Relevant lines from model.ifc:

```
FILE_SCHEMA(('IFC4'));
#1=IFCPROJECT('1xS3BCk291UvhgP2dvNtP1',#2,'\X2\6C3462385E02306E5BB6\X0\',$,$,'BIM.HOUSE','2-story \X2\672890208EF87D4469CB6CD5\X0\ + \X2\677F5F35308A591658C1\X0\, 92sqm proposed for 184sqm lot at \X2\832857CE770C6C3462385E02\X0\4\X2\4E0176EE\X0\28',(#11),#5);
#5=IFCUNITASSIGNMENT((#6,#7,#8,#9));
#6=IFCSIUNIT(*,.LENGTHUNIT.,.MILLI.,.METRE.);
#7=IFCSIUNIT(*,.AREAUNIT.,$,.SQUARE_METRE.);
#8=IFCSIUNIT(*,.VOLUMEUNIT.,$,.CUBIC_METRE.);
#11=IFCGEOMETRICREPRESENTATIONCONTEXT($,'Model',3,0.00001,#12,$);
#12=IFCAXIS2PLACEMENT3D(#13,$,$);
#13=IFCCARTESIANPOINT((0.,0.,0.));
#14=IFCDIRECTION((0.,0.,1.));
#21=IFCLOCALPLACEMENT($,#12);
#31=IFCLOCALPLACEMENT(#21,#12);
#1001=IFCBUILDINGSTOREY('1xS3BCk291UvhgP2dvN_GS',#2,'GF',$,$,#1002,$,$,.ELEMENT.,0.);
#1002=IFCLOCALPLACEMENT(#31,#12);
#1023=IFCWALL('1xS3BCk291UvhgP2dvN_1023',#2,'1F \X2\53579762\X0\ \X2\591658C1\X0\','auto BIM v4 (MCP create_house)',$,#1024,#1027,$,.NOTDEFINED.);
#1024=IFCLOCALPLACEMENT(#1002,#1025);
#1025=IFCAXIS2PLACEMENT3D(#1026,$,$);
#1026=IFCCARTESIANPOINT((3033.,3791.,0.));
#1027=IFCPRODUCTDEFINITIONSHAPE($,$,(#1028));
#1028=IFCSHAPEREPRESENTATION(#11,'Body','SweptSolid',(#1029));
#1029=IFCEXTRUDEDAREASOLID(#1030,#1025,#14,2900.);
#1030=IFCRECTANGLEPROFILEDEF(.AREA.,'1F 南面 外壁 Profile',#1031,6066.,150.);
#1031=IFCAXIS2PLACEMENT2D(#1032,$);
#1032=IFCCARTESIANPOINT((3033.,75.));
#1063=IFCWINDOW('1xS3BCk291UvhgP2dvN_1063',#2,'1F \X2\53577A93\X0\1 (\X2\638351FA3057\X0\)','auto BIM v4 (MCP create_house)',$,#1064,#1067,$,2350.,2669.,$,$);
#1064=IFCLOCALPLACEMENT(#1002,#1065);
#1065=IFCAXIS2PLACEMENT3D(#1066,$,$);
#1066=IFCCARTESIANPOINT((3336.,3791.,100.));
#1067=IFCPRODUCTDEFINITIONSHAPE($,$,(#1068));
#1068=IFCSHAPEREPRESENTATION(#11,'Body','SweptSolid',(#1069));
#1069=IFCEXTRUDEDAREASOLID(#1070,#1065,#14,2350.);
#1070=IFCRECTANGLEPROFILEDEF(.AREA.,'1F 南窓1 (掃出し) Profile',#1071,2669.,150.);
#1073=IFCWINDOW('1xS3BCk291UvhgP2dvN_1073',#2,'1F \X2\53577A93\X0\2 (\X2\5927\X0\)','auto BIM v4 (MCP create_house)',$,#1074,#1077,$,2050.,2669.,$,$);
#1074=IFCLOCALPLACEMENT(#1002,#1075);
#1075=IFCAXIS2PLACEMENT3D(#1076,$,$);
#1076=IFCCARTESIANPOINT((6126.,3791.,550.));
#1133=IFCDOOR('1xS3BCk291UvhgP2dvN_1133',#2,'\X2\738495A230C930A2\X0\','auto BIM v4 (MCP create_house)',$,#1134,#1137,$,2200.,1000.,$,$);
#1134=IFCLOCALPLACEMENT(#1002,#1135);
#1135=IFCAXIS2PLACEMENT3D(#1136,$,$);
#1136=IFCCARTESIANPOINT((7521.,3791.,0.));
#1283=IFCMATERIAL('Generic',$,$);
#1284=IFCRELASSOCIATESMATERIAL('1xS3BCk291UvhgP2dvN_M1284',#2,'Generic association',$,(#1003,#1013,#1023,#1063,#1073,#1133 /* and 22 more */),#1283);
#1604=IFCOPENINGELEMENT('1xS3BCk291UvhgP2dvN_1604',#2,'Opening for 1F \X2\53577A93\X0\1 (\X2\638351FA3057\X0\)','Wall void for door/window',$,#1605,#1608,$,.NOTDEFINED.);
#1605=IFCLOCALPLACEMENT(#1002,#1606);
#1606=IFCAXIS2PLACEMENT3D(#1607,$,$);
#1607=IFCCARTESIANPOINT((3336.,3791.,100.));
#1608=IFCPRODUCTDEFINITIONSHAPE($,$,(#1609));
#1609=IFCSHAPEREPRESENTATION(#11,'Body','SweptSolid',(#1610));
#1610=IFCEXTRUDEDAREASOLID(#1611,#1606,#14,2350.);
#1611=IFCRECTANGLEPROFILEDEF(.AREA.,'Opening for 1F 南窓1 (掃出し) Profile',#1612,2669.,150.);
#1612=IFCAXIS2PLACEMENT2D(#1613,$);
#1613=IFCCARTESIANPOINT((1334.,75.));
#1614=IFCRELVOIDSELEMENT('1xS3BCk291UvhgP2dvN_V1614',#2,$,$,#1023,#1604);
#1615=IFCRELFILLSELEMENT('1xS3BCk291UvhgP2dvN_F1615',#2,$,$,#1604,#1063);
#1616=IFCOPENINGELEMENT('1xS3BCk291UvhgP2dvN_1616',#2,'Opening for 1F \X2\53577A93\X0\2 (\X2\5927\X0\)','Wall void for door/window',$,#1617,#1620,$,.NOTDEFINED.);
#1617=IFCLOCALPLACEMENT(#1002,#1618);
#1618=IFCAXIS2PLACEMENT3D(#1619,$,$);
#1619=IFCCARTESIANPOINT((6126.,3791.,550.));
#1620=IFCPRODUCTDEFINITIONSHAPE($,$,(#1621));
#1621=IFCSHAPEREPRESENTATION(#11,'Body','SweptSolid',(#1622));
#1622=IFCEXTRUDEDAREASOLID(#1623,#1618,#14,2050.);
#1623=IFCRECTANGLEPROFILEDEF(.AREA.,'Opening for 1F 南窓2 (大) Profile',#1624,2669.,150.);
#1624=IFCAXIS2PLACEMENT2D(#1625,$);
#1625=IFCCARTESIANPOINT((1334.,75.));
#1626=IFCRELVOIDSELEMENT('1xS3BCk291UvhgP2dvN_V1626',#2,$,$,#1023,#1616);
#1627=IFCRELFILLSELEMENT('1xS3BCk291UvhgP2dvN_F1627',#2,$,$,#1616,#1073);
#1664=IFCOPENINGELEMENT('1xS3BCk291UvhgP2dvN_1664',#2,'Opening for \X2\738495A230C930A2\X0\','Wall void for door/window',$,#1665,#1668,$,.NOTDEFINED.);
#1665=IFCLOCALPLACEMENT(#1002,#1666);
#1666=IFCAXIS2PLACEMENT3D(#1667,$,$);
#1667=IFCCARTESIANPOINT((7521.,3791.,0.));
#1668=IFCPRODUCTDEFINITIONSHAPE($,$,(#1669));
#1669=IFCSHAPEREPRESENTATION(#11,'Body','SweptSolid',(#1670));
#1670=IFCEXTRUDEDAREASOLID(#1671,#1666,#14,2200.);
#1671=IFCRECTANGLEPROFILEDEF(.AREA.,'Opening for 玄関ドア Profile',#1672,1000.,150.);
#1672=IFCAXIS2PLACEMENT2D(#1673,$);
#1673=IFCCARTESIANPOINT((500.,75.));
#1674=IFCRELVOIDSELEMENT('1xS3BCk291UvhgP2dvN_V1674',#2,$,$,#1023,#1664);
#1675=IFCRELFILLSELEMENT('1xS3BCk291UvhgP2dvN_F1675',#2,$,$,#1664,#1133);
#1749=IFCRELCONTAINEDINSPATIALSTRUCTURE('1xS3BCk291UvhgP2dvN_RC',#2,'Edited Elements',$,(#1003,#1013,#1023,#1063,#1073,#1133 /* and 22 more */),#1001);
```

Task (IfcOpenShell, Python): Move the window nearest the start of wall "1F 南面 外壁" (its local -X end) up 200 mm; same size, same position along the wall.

```python
import numpy as np
import ifcopenshell
import ifcopenshell.api.geometry
import ifcopenshell.util.placement
import ifcopenshell.util.unit

model = ifcopenshell.open("model.ifc")
unit_scale = ifcopenshell.util.unit.calculate_unit_scale(model)

window = model.by_guid("1xS3BCk291UvhgP2dvN_1063")
opening = window.FillsVoids[0].RelatingOpeningElement
dz = 0.2 / unit_scale

shift = np.array([0.0, 0.0, dz])
# The window is not placed relative to its opening, so move both.
for product in (opening, window):
    matrix = ifcopenshell.util.placement.get_local_placement(product.ObjectPlacement)
    matrix[:3, 3] += shift
    ifcopenshell.api.geometry.edit_object_placement(model, product=product, matrix=matrix, is_si=False)

print(f"moved by {dz * unit_scale:+.3f} m")

model.write("model_updated.ifc")
```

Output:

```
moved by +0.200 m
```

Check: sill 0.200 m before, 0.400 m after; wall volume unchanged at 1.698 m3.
